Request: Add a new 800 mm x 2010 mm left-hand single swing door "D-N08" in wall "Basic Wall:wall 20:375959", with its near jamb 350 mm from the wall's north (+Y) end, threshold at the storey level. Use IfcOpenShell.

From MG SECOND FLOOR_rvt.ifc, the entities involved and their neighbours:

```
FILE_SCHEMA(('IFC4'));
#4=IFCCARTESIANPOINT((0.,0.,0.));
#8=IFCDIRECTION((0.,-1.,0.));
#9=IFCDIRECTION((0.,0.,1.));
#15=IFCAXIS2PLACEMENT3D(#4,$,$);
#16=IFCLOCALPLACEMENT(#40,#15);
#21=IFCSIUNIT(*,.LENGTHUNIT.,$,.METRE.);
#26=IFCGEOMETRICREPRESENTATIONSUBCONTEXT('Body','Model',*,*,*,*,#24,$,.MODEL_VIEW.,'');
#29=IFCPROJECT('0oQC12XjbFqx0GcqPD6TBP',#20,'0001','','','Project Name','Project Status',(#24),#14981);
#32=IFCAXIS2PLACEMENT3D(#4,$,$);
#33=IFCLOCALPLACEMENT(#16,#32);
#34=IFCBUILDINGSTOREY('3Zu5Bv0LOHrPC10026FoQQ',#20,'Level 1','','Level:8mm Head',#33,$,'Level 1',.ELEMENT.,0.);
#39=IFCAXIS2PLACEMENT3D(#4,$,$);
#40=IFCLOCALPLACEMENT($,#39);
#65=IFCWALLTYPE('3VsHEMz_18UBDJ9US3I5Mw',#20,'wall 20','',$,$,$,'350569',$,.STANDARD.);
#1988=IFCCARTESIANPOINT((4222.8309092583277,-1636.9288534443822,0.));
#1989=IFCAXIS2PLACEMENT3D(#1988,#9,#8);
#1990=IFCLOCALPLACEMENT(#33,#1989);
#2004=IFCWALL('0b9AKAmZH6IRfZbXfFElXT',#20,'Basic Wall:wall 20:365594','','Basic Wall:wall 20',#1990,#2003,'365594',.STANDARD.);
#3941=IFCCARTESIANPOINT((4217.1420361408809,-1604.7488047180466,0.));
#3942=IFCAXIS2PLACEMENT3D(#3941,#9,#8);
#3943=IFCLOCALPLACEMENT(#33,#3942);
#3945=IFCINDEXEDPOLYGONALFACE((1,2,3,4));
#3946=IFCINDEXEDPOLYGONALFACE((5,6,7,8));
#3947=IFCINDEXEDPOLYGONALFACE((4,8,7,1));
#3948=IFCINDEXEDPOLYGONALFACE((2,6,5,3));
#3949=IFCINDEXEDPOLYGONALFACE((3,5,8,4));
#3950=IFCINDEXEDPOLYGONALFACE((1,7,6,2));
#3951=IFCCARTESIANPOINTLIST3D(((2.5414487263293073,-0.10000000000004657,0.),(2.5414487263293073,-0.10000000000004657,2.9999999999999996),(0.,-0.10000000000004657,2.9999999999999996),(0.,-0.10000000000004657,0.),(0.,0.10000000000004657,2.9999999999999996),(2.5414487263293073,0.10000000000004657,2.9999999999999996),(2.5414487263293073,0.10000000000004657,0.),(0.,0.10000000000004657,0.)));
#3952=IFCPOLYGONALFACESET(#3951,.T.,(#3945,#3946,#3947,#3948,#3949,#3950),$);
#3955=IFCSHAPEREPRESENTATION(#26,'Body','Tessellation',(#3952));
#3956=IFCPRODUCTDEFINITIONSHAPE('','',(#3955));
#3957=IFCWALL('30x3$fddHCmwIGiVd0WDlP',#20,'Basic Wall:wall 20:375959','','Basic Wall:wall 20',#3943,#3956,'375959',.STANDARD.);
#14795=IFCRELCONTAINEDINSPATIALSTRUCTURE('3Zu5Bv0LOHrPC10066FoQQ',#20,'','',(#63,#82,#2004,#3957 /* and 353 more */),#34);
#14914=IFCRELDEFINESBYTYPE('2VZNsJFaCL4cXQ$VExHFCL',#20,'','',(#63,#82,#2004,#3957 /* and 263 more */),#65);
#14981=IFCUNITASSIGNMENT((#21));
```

```python
import numpy as np
import ifcopenshell
import ifcopenshell.api.feature
import ifcopenshell.api.geometry
import ifcopenshell.api.root
import ifcopenshell.api.spatial
import ifcopenshell.geom
import ifcopenshell.util.element
import ifcopenshell.util.placement
import ifcopenshell.util.representation
import ifcopenshell.util.shape
import ifcopenshell.util.unit

model = ifcopenshell.open("MG SECOND FLOOR_rvt.ifc")
unit_scale = ifcopenshell.util.unit.calculate_unit_scale(model)
settings = ifcopenshell.geom.settings()


def volume(element):
    """Net volume in cubic metres, openings subtracted."""
    shape = ifcopenshell.geom.create_shape(settings, element)
    return ifcopenshell.util.shape.get_volume(shape.geometry)


wall = model.by_guid("30x3$fddHCmwIGiVd0WDlP")
storey = ifcopenshell.util.element.get_container(wall, ifc_class="IfcBuildingStorey")
context = ifcopenshell.util.representation.get_context(model, "Model", "Body", "MODEL_VIEW")
before = volume(wall)

width, height, from_end, sill = 0.8, 2.01, 0.35, 0.0  # metres

# The wall runs along its own X axis, and the end named is its -X end.
wall_shape = ifcopenshell.geom.create_shape(settings, wall)
x, y, z = ifcopenshell.util.shape.get_vertices(wall_shape.geometry).T
start = x.min() + from_end
face, thickness = float(y.min()), float(y.max() - y.min())
wall_matrix = ifcopenshell.util.placement.get_local_placement(wall.ObjectPlacement)
level = ifcopenshell.util.placement.get_local_placement(storey.ObjectPlacement)[2, 3]


def in_wall(x, y):
    """Placement at x, y metres in the wall's axes, at sill height."""
    matrix = wall_matrix.copy()
    matrix[:, 3] = wall_matrix @ np.array([x / unit_scale, y / unit_scale, 0.0, 1.0])
    matrix[2, 3] = level + sill / unit_scale
    return matrix


# Opening: a box that overshoots both wall faces by 50 mm.
opening = ifcopenshell.api.root.create_entity(model, ifc_class="IfcOpeningElement", predefined_type="OPENING")
box = ifcopenshell.api.geometry.add_wall_representation(
    model, context=context, length=width, height=height, thickness=thickness + 0.1
)
ifcopenshell.api.geometry.assign_representation(model, product=opening, representation=box)
ifcopenshell.api.geometry.edit_object_placement(model, product=opening, matrix=in_wall(start, face - 0.05), is_si=False)
ifcopenshell.api.feature.add_feature(model, feature=opening, element=wall)

door = ifcopenshell.api.root.create_entity(model, ifc_class="IfcDoor", name="D-N08", predefined_type="DOOR")
door.OverallWidth, door.OverallHeight = width / unit_scale, height / unit_scale
door.OperationType = "SINGLE_SWING_LEFT"
body = ifcopenshell.api.geometry.add_door_representation(
    model,
    context=context,
    overall_width=door.OverallWidth,
    overall_height=door.OverallHeight,
    operation_type="SINGLE_SWING_LEFT",
    lining_properties={"LiningDepth": thickness / unit_scale, "ThresholdDepth": thickness / unit_scale},
)
ifcopenshell.api.geometry.assign_representation(model, product=door, representation=body)
ifcopenshell.api.spatial.assign_container(model, products=[door], relating_structure=storey)
ifcopenshell.api.feature.add_filling(model, opening=opening, element=door)

# The lining spans the wall, so the door starts at the wall face.
ifcopenshell.api.geometry.edit_object_placement(model, product=door, matrix=in_wall(start, face), is_si=False)

after = volume(wall)

print(f"wall volume {before:.3f} -> {after:.3f} m3")

model.write("MG SECOND FLOOR_rvt_edited.ifc")
```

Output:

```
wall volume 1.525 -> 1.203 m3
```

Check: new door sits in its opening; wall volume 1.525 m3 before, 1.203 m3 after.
